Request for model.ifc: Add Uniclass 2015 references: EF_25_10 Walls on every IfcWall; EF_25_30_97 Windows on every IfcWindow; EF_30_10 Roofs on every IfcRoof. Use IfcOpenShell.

First a look at what the model holds.

```python
import ifcopenshell

model = ifcopenshell.open("model.ifc")
print(model.schema)
print("classifications:", [c.Name for c in model.by_type("IfcClassification")])
for ifc_class in ("IfcDoor", "IfcRoof", "IfcStair", "IfcWall", "IfcWindow"):
    print(ifc_class, len(model.by_type(ifc_class)))
```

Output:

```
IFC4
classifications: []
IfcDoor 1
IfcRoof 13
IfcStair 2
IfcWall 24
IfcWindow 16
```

```python
import ifcopenshell
import ifcopenshell.api.classification

model = ifcopenshell.open("model.ifc")

system = ifcopenshell.api.classification.add_classification(model, classification="Uniclass 2015")

codes = {
    "IfcWall": ("EF_25_10", "Walls"),
    "IfcWindow": ("EF_25_30_97", "Windows"),
    "IfcRoof": ("EF_30_10", "Roofs"),
}
for ifc_class, (code, name) in codes.items():
    products = model.by_type(ifc_class)
    ifcopenshell.api.classification.add_reference(
        model, products=products, classification=system, identification=code, name=name
    )
    print(code, len(products))

model.write("model-out.ifc")
```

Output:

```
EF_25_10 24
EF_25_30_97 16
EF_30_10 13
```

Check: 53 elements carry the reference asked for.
